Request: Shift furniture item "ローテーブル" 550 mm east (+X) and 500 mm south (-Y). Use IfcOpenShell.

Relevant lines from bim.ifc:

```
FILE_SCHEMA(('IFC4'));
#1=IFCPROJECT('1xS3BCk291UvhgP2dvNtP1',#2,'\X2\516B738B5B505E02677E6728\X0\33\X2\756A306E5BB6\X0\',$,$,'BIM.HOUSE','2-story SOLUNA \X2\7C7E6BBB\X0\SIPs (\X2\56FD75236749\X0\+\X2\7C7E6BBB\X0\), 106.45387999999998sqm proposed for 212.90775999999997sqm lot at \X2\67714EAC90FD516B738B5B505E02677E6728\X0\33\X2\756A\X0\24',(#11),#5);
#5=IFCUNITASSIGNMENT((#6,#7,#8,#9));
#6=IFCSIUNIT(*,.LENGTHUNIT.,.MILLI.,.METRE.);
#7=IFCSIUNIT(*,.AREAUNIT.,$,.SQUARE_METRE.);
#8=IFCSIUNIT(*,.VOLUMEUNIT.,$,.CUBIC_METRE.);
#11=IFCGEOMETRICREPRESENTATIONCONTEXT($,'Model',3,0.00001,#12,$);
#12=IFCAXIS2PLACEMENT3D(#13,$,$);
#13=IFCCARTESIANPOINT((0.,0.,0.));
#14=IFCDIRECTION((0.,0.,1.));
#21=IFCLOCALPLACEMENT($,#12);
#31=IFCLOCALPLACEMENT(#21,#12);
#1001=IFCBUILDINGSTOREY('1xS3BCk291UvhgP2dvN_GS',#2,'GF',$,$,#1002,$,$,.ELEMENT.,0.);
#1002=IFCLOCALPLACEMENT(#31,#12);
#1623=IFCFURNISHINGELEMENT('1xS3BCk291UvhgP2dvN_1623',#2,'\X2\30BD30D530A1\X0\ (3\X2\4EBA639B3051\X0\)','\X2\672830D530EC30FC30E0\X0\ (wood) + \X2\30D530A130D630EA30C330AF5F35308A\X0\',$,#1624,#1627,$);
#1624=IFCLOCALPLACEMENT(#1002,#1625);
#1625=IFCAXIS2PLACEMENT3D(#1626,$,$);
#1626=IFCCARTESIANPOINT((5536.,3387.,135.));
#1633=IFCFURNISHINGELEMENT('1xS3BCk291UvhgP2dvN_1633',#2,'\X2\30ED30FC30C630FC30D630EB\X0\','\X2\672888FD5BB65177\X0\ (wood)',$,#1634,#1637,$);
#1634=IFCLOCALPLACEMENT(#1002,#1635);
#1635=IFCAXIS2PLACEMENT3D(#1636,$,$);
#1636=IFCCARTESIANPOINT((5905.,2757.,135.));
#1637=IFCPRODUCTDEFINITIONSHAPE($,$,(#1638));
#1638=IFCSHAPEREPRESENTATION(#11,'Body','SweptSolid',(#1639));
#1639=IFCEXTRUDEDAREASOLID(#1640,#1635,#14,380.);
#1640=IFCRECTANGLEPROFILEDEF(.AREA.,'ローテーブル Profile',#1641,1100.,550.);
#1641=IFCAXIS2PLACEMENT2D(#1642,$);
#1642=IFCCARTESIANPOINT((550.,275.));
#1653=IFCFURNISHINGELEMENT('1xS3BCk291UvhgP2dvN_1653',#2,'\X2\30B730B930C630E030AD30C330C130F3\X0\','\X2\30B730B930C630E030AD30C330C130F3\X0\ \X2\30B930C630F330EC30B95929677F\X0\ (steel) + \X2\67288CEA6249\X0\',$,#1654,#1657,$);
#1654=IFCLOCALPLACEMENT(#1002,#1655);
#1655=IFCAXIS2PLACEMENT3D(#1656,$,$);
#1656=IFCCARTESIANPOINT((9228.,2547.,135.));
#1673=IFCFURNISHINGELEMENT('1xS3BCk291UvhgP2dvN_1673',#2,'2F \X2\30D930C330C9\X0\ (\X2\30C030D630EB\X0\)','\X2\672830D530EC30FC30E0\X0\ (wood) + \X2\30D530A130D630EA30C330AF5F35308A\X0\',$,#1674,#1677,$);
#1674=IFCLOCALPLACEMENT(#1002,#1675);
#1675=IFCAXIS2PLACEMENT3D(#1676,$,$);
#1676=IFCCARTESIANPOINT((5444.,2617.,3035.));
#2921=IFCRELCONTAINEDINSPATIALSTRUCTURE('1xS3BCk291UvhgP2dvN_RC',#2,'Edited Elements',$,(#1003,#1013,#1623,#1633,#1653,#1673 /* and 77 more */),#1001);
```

```python
import ifcopenshell
import ifcopenshell.api.geometry
import ifcopenshell.util.placement

model = ifcopenshell.open("bim.ifc")

item = model.by_id(1633)
matrix = ifcopenshell.util.placement.get_local_placement(item.ObjectPlacement)
matrix[0, 3] += 550.0
matrix[1, 3] -= 500.0
ifcopenshell.api.geometry.edit_object_placement(model, product=item, matrix=matrix, is_si=False)

print(ifcopenshell.util.placement.get_local_placement(item.ObjectPlacement).round(3) + 0.0)

model.write("bim-out.ifc")
```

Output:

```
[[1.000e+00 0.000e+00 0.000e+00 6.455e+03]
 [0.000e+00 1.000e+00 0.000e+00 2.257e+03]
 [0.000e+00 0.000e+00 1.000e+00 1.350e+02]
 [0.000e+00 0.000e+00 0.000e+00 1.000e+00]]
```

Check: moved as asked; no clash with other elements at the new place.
